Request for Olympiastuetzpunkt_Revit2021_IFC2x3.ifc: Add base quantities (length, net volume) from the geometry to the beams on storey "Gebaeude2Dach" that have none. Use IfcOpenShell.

First a look at what the model holds.

```python
import ifcopenshell
import ifcopenshell.util.element
import ifcopenshell.util.unit

model = ifcopenshell.open("Olympiastuetzpunkt_Revit2021_IFC2x3.ifc")
print(model.schema)
for unit_type in ("LENGTHUNIT", "AREAUNIT", "VOLUMEUNIT"):
    print(unit_type, ifcopenshell.util.unit.calculate_unit_scale(model, unit_type))
storey = next(s for s in model.by_type("IfcBuildingStorey") if s.Name == "Gebaeude2Dach")
beams = [e for e in ifcopenshell.util.element.get_decomposition(storey) if e.is_a("IfcBeam")]
for e in sorted(beams, key=lambda e: e.id()):
    print(e.id(), e.is_a(), e.Name, list(ifcopenshell.util.element.get_psets(e, qtos_only=True)), sep=" | ")
```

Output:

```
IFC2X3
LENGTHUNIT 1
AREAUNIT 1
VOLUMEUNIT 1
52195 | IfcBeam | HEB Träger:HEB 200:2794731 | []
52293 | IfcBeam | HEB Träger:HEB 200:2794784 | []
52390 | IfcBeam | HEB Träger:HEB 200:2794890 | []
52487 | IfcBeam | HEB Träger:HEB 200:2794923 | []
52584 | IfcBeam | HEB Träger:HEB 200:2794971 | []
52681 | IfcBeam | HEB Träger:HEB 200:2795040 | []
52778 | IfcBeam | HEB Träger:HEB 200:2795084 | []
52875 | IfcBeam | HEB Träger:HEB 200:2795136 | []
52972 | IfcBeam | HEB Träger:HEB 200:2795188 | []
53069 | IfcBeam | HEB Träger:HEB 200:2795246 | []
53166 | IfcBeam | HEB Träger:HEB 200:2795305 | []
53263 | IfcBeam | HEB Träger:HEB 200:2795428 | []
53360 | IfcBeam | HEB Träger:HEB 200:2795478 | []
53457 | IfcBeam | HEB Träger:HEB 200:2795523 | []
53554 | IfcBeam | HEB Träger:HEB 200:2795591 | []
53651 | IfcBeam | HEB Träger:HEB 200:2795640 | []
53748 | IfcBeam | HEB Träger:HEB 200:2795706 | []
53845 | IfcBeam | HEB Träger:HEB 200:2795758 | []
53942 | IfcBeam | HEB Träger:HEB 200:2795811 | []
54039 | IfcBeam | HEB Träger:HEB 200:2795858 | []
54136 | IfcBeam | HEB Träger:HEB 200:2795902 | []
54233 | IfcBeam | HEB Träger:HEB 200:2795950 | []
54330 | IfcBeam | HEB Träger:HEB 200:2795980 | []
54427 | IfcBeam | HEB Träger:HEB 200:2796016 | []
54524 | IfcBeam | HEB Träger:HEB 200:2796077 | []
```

```python
import ifcopenshell
import ifcopenshell.api.pset
import ifcopenshell.geom
import ifcopenshell.util.element
import ifcopenshell.util.shape
import ifcopenshell.util.unit

model = ifcopenshell.open("Olympiastuetzpunkt_Revit2021_IFC2x3.ifc")
unit_scale = ifcopenshell.util.unit.calculate_unit_scale(model)
volume_scale = ifcopenshell.util.unit.calculate_unit_scale(model, "VOLUMEUNIT")
settings = ifcopenshell.geom.settings()

storey = next(s for s in model.by_type("IfcBuildingStorey") if s.Name == "Gebaeude2Dach")
beams = [e for e in ifcopenshell.util.element.get_decomposition(storey) if e.is_a("IfcBeam")]

for e in sorted(beams, key=lambda e: e.id()):
    if ifcopenshell.util.element.get_psets(e, qtos_only=True, should_inherit=False):
        continue
    # Geometry comes back in metres, in the element's own axes.
    shape = ifcopenshell.geom.create_shape(settings, e)
    values = {
        "Length": ifcopenshell.util.shape.get_max_xyz(shape.geometry) / unit_scale,
        "NetVolume": ifcopenshell.util.shape.get_volume(shape.geometry) / volume_scale,
    }
    qto = ifcopenshell.api.pset.add_qto(model, product=e, name="BaseQuantities")
    ifcopenshell.api.pset.edit_qto(model, qto=qto, properties=values)
    print(e.id(), {k: round(v, 3) for k, v in values.items()})

model.write("Olympiastuetzpunkt_Revit2021_IFC2x3_rev.ifc")
```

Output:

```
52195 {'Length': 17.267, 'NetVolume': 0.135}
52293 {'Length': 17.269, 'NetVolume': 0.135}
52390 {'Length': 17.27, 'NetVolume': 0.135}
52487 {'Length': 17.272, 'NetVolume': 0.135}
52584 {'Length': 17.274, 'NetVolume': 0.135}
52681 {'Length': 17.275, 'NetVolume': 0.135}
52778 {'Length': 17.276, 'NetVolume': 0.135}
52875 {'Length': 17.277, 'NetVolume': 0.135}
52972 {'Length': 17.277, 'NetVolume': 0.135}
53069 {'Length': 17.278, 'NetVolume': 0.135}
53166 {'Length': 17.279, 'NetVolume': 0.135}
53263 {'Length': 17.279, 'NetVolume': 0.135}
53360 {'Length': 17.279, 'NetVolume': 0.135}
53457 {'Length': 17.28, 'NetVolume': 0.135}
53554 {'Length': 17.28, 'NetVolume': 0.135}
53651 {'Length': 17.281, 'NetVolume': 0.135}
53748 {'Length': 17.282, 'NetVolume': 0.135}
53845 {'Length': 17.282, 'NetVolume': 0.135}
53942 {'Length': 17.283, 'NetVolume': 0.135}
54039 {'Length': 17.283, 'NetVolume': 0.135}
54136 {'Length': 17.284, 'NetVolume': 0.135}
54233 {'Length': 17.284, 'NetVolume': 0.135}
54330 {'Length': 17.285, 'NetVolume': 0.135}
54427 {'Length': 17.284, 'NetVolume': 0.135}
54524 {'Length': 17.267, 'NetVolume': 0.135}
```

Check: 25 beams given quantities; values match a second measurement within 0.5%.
